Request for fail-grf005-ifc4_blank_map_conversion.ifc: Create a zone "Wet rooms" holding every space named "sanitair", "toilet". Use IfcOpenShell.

First a look at what the model holds.

```python
import ifcopenshell

model = ifcopenshell.open("fail-grf005-ifc4_blank_map_conversion.ifc")
print(model.schema)
seen = {}
for space in model.by_type("IfcSpace"):
    seen[space.LongName] = seen.get(space.LongName, 0) + 1
for name, count in sorted(seen.items(), key=str):
    print(count, "x", name)
print("zones:", [z.Name for z in model.by_type("IfcZone")][:20])
```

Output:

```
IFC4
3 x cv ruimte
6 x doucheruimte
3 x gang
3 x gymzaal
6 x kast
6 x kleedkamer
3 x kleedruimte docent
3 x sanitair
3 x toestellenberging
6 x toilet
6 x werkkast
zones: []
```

```python
import ifcopenshell
import ifcopenshell.api.group
import ifcopenshell.api.root

model = ifcopenshell.open("fail-grf005-ifc4_blank_map_conversion.ifc")

names = {"sanitair", "toilet"}
spaces = [s for s in model.by_type("IfcSpace") if s.LongName in names]

zone = ifcopenshell.api.root.create_entity(model, ifc_class="IfcZone", name="Wet rooms")
ifcopenshell.api.group.assign_group(model, products=spaces, group=zone)
print(len(spaces), "spaces in", zone.Name)

model.write("fail-grf005-ifc4_blank_map_conversion_v2.ifc")
```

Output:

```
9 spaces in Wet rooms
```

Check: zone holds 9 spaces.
